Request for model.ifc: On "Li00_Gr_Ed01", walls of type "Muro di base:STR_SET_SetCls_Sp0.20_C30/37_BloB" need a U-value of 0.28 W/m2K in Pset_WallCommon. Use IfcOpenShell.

First a look at what the model holds.

```python
import ifcopenshell
import ifcopenshell.util.element

model = ifcopenshell.open("model.ifc")
print(model.schema)
storey = next(s for s in model.by_type("IfcBuildingStorey") if s.Name == "Li00_Gr_Ed01")
walls = [e for e in ifcopenshell.util.element.get_decomposition(storey) if e.is_a("IfcWall")]
seen = {}
for e in walls:
    element_type = ifcopenshell.util.element.get_type(e)
    key = (element_type.Name if element_type != e and element_type else None, ifcopenshell.util.element.get_pset(e, "Pset_WallCommon", "ThermalTransmittance"))
    seen[key] = seen.get(key, 0) + 1
for (name, value), count in sorted(seen.items(), key=str):
    print(count, "x", name, "|", value)
```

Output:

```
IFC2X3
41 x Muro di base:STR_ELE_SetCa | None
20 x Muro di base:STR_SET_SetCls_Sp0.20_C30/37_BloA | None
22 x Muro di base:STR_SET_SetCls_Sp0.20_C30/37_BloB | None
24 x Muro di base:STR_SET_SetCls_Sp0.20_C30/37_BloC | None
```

```python
import ifcopenshell
import ifcopenshell.api.pset
import ifcopenshell.util.element

model = ifcopenshell.open("model.ifc")

storey = next(s for s in model.by_type("IfcBuildingStorey") if s.Name == "Li00_Gr_Ed01")
walls = [e for e in ifcopenshell.util.element.get_decomposition(storey) if e.is_a("IfcWall")]

count = 0
for e in walls:
    element_type = ifcopenshell.util.element.get_type(e)
    if element_type in (None, e) or element_type.Name != "Muro di base:STR_SET_SetCls_Sp0.20_C30/37_BloB":
        continue
    # add_pset returns the element's existing set when there is one.
    pset = ifcopenshell.api.pset.add_pset(model, product=e, name="Pset_WallCommon")
    ifcopenshell.api.pset.edit_pset(model, pset=pset, properties={"ThermalTransmittance": 0.28})
    count += 1

print(count, "walls updated")

model.write("model_edited.ifc")
```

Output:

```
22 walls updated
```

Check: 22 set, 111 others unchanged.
